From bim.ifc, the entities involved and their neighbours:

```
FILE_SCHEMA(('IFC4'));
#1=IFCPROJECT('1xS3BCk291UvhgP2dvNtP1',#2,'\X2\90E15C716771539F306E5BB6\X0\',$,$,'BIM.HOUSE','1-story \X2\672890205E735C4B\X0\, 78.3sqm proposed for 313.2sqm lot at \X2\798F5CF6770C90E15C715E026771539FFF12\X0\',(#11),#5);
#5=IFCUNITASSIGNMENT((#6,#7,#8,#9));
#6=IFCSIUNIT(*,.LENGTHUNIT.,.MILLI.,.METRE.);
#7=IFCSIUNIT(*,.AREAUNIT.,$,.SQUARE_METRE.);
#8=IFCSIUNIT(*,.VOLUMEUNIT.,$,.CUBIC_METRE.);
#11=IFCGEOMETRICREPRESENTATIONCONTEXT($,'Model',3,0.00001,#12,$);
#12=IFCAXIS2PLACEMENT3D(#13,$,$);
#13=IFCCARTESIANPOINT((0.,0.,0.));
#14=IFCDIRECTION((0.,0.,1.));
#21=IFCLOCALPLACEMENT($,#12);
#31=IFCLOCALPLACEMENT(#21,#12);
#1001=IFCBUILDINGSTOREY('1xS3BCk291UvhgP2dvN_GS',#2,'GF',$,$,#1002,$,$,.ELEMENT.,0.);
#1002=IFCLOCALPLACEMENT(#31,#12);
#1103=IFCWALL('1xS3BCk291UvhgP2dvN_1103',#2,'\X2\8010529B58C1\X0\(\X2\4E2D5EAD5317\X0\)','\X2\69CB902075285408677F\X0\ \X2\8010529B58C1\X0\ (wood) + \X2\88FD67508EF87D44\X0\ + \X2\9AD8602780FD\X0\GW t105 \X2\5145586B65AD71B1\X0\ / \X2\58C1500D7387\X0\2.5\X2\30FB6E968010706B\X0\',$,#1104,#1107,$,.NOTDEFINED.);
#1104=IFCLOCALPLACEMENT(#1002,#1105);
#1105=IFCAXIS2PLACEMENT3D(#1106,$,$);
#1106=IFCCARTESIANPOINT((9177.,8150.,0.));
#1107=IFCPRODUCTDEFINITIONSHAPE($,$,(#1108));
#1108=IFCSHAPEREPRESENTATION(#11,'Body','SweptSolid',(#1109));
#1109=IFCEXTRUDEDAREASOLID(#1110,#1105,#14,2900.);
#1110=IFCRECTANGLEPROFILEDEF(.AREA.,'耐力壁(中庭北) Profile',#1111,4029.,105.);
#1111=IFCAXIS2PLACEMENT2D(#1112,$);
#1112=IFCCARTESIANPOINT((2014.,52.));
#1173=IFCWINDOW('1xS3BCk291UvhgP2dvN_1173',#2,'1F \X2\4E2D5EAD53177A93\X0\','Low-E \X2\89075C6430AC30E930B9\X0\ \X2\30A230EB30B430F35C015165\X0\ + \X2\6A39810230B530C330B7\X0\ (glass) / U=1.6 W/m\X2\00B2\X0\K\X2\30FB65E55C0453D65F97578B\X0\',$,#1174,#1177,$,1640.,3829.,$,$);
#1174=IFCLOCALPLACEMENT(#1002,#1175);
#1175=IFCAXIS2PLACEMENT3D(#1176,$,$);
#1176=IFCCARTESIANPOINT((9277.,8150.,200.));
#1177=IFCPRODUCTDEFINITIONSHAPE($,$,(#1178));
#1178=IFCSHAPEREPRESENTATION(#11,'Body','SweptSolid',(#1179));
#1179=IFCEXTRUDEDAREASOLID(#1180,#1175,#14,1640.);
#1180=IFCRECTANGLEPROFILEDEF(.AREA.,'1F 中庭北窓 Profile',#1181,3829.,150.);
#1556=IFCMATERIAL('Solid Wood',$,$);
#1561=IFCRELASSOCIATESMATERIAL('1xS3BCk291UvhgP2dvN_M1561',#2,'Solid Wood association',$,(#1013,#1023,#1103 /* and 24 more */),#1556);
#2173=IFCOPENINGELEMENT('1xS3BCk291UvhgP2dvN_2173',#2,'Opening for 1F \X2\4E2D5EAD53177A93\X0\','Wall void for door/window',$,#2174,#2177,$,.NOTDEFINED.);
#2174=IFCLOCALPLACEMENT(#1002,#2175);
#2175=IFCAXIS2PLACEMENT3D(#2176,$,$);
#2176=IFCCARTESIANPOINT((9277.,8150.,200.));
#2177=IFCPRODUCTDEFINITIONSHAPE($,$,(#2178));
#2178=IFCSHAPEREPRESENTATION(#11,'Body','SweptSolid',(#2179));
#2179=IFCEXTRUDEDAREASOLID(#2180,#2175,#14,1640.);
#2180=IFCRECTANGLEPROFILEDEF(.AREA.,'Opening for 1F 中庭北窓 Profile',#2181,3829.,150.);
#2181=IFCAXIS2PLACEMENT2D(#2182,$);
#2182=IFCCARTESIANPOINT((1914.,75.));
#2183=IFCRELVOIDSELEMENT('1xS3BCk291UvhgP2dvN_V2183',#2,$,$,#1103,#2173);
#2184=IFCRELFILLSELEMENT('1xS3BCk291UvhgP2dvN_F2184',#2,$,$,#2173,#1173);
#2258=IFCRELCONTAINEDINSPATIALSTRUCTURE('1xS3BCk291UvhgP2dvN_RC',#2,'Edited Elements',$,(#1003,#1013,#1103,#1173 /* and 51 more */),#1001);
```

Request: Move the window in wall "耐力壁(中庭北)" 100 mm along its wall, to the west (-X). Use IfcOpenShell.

```python
import ifcopenshell
import ifcopenshell.api.geometry
import ifcopenshell.util.placement
import ifcopenshell.util.unit

model = ifcopenshell.open("bim.ifc")
unit_scale = ifcopenshell.util.unit.calculate_unit_scale(model)

window = model.by_guid("1xS3BCk291UvhgP2dvN_1173")
opening = window.FillsVoids[0].RelatingOpeningElement
wall = opening.VoidsElements[0].RelatingBuildingElement

wall_matrix = ifcopenshell.util.placement.get_local_placement(wall.ObjectPlacement)
shift = wall_matrix[:3, 0] * -0.1 / unit_scale
before = ifcopenshell.util.placement.get_local_placement(window.ObjectPlacement)[:3, 3].copy()

# The window is not placed relative to its opening, so move both.
for product in (opening, window):
    matrix = ifcopenshell.util.placement.get_local_placement(product.ObjectPlacement)
    matrix[:3, 3] += shift
    ifcopenshell.api.geometry.edit_object_placement(model, product=product, matrix=matrix, is_si=False)

after = ifcopenshell.util.placement.get_local_placement(window.ObjectPlacement)[:3, 3]
print("window moved by", (after - before).round(3) + 0.0)

model.write("bim_edited.ifc")
```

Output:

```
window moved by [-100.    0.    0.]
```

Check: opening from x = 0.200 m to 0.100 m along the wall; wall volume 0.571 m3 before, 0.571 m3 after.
